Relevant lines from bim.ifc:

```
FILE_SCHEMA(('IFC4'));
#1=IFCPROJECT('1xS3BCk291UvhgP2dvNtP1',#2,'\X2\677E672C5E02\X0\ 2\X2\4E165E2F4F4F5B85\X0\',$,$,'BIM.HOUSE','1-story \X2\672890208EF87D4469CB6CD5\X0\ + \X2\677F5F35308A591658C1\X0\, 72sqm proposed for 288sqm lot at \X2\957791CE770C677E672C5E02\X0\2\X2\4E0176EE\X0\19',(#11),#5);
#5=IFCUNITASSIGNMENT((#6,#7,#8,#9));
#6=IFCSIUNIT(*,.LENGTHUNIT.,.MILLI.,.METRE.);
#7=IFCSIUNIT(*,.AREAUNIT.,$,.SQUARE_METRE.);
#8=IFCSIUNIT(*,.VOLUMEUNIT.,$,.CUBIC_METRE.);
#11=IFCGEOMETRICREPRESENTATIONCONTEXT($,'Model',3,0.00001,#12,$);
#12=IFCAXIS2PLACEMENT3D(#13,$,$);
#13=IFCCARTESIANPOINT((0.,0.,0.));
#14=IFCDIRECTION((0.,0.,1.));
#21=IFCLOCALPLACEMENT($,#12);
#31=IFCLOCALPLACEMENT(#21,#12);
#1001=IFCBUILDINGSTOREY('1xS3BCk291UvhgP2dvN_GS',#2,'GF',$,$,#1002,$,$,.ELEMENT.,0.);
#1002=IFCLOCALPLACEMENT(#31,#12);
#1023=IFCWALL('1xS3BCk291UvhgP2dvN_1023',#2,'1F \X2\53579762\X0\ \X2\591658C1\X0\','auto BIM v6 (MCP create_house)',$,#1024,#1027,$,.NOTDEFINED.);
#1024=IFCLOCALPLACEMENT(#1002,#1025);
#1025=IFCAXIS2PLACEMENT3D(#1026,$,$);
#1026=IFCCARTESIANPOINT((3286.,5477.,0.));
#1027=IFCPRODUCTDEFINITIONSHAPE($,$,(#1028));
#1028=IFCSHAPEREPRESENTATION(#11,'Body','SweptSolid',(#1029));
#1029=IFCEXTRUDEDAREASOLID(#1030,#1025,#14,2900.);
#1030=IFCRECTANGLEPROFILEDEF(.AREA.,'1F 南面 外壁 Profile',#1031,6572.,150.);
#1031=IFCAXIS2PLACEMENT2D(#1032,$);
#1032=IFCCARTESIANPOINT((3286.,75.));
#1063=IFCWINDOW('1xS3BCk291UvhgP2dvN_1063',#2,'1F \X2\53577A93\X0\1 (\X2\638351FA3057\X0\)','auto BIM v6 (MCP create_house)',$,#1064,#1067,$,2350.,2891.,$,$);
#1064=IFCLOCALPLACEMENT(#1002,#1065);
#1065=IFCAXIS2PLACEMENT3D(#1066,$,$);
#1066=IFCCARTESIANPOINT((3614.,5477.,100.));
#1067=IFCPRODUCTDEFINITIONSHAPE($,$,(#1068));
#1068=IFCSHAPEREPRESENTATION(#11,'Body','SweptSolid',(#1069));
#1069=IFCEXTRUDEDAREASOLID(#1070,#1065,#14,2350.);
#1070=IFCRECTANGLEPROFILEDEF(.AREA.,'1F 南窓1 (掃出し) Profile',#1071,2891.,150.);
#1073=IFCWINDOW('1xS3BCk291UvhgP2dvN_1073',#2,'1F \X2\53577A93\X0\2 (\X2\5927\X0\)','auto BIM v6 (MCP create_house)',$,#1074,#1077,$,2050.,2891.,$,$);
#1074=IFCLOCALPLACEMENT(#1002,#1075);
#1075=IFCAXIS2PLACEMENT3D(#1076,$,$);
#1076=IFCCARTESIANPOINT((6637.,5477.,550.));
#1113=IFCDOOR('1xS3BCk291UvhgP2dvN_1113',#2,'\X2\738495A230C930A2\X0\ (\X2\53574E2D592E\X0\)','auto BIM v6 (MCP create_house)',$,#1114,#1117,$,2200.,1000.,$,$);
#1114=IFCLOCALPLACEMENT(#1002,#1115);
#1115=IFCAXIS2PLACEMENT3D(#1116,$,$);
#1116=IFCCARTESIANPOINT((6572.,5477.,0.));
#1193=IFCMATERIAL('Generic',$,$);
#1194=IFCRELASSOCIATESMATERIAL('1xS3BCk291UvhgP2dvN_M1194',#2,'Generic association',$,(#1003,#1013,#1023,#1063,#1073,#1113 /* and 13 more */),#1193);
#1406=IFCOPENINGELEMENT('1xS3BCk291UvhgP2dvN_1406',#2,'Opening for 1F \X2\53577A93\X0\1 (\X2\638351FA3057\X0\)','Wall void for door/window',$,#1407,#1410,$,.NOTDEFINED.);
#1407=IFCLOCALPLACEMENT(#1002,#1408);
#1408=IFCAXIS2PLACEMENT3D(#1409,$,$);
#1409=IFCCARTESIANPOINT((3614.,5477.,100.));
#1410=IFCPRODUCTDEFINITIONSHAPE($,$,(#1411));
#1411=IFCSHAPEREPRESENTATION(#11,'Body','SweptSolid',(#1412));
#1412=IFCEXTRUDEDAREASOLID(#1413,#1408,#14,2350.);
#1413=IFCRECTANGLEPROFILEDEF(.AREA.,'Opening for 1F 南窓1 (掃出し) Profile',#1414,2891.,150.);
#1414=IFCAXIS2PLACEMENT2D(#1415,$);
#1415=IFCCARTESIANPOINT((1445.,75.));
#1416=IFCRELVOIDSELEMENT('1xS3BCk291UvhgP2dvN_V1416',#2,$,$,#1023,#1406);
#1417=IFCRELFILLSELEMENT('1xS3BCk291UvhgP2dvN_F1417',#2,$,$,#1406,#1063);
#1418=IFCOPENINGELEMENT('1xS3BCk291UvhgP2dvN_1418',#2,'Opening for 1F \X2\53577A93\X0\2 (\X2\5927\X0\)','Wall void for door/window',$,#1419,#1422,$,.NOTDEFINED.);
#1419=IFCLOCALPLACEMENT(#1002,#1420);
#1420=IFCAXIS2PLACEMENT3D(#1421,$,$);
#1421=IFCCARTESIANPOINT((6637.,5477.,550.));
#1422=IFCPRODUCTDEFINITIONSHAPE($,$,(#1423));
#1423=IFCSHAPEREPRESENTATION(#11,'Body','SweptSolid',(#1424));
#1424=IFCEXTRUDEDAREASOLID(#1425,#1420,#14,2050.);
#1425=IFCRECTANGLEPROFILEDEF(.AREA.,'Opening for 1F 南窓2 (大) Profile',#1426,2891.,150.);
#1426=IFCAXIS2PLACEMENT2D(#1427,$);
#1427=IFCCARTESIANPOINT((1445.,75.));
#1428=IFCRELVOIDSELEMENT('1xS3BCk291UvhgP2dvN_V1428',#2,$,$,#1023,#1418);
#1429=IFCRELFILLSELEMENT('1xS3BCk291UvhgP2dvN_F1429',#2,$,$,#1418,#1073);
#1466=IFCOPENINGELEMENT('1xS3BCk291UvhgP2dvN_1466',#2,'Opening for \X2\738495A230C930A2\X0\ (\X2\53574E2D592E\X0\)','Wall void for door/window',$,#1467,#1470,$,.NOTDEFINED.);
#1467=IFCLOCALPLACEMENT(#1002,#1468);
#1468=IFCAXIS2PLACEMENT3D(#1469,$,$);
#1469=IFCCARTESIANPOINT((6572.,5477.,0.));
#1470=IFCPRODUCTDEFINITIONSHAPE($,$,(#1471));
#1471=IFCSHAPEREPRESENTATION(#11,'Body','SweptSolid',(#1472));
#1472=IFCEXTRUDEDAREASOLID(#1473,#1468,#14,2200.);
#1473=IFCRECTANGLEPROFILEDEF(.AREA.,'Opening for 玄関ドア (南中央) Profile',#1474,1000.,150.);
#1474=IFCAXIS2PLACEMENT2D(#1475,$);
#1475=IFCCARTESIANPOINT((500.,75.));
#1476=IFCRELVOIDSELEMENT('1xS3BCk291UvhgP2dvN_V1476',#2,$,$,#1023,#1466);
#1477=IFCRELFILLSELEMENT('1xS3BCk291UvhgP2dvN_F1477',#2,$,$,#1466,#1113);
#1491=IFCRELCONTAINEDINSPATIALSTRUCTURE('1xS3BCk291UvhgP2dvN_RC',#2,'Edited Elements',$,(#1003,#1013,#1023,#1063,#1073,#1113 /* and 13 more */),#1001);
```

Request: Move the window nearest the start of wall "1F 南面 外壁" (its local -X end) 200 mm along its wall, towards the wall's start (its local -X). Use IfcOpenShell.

```python
import ifcopenshell
import ifcopenshell.api.geometry
import ifcopenshell.util.placement
import ifcopenshell.util.unit

model = ifcopenshell.open("bim.ifc")
unit_scale = ifcopenshell.util.unit.calculate_unit_scale(model)

window = model.by_guid("1xS3BCk291UvhgP2dvN_1063")
opening = window.FillsVoids[0].RelatingOpeningElement
wall = opening.VoidsElements[0].RelatingBuildingElement

wall_matrix = ifcopenshell.util.placement.get_local_placement(wall.ObjectPlacement)
shift = wall_matrix[:3, 0] * -0.2 / unit_scale
before = ifcopenshell.util.placement.get_local_placement(window.ObjectPlacement)[:3, 3].copy()

# The window is not placed relative to its opening, so move both.
for product in (opening, window):
    matrix = ifcopenshell.util.placement.get_local_placement(product.ObjectPlacement)
    matrix[:3, 3] += shift
    ifcopenshell.api.geometry.edit_object_placement(model, product=product, matrix=matrix, is_si=False)

after = ifcopenshell.util.placement.get_local_placement(window.ObjectPlacement)[:3, 3]
print("window moved by", (after - before).round(3) + 0.0)

model.write("bim_rev.ifc")
```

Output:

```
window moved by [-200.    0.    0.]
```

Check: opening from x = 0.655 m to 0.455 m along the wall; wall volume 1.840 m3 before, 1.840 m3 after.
